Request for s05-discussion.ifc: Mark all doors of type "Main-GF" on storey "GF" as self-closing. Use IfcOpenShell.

First a look at what the model holds.

```python
import ifcopenshell
import ifcopenshell.util.element

model = ifcopenshell.open("s05-discussion.ifc")
print(model.schema)
storey = next(s for s in model.by_type("IfcBuildingStorey") if s.Name == "GF")
doors = [e for e in ifcopenshell.util.element.get_decomposition(storey) if e.is_a("IfcDoor")]
seen = {}
for e in doors:
    element_type = ifcopenshell.util.element.get_type(e)
    key = (element_type.Name if element_type != e and element_type else None, ifcopenshell.util.element.get_pset(e, "Pset_DoorCommon", "SelfClosing"))
    seen[key] = seen.get(key, 0) + 1
for (name, value), count in sorted(seen.items(), key=str):
    print(count, "x", name, "|", value)
```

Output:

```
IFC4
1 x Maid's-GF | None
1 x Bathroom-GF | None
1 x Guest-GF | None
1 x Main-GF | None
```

```python
import ifcopenshell
import ifcopenshell.api.pset
import ifcopenshell.util.element

model = ifcopenshell.open("s05-discussion.ifc")

storey = next(s for s in model.by_type("IfcBuildingStorey") if s.Name == "GF")
doors = [e for e in ifcopenshell.util.element.get_decomposition(storey) if e.is_a("IfcDoor")]

count = 0
for e in doors:
    element_type = ifcopenshell.util.element.get_type(e)
    if element_type in (None, e) or element_type.Name != "Main-GF":
        continue
    # add_pset returns the element's existing set when there is one.
    pset = ifcopenshell.api.pset.add_pset(model, product=e, name="Pset_DoorCommon")
    ifcopenshell.api.pset.edit_pset(model, pset=pset, properties={"SelfClosing": True})
    count += 1

print(count, "doors updated")

model.write("s05-discussion_rev.ifc")
```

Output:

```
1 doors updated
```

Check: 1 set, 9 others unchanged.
